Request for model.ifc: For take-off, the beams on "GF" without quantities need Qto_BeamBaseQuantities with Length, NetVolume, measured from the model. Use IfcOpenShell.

First a look at what the model holds.

```python
import ifcopenshell
import ifcopenshell.util.element
import ifcopenshell.util.unit

model = ifcopenshell.open("model.ifc")
print(model.schema)
for unit_type in ("LENGTHUNIT", "AREAUNIT", "VOLUMEUNIT"):
    print(unit_type, ifcopenshell.util.unit.calculate_unit_scale(model, unit_type))
storey = next(s for s in model.by_type("IfcBuildingStorey") if s.Name == "GF")
beams = [e for e in ifcopenshell.util.element.get_decomposition(storey) if e.is_a("IfcBeam")]
for e in sorted(beams, key=lambda e: e.id()):
    print(e.id(), e.is_a(), e.Name, list(ifcopenshell.util.element.get_psets(e, qtos_only=True)), sep=" | ")
```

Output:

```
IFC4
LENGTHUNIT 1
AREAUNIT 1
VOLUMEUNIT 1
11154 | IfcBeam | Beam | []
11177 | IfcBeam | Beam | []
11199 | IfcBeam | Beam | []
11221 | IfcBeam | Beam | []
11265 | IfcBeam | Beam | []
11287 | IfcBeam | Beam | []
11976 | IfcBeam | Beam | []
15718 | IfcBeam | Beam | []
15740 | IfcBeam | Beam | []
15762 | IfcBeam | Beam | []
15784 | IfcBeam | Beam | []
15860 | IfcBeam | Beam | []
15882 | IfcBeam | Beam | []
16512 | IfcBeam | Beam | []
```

```python
import ifcopenshell
import ifcopenshell.api.pset
import ifcopenshell.geom
import ifcopenshell.util.element
import ifcopenshell.util.shape
import ifcopenshell.util.unit

model = ifcopenshell.open("model.ifc")
unit_scale = ifcopenshell.util.unit.calculate_unit_scale(model)
volume_scale = ifcopenshell.util.unit.calculate_unit_scale(model, "VOLUMEUNIT")
settings = ifcopenshell.geom.settings()

storey = next(s for s in model.by_type("IfcBuildingStorey") if s.Name == "GF")
beams = [e for e in ifcopenshell.util.element.get_decomposition(storey) if e.is_a("IfcBeam")]

for e in sorted(beams, key=lambda e: e.id()):
    if ifcopenshell.util.element.get_psets(e, qtos_only=True, should_inherit=False):
        continue
    # Geometry comes back in metres, in the element's own axes.
    shape = ifcopenshell.geom.create_shape(settings, e)
    values = {
        "Length": ifcopenshell.util.shape.get_max_xyz(shape.geometry) / unit_scale,
        "NetVolume": ifcopenshell.util.shape.get_volume(shape.geometry) / volume_scale,
    }
    qto = ifcopenshell.api.pset.add_qto(model, product=e, name="Qto_BeamBaseQuantities")
    ifcopenshell.api.pset.edit_qto(model, qto=qto, properties=values)
    print(e.id(), {k: round(v, 3) for k, v in values.items()})

model.write("model_edited.ifc")
```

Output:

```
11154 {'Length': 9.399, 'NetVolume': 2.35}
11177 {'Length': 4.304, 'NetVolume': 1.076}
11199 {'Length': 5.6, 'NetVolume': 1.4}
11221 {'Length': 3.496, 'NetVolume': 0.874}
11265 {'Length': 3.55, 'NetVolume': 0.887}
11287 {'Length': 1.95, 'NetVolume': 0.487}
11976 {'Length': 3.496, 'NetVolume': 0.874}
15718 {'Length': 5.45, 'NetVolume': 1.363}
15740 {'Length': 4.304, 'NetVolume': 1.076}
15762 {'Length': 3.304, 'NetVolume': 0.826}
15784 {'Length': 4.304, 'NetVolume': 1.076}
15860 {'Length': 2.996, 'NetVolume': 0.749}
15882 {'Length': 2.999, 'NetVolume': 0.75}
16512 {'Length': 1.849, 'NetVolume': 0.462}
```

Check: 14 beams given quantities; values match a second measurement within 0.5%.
